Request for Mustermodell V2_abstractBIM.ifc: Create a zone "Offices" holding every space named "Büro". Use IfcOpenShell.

First a look at what the model holds.

```python
import ifcopenshell

model = ifcopenshell.open("Mustermodell V2_abstractBIM.ifc")
print(model.schema)
seen = {}
for space in model.by_type("IfcSpace"):
    seen[space.LongName] = seen.get(space.LongName, 0) + 1
for name, count in sorted(seen.items(), key=str):
    print(count, "x", name)
print("zones:", [z.Name for z in model.by_type("IfcZone")][:20])
```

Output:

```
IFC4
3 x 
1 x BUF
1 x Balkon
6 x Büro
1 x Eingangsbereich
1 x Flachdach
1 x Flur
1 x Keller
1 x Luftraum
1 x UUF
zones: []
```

```python
import ifcopenshell
import ifcopenshell.api.group
import ifcopenshell.api.root

model = ifcopenshell.open("Mustermodell V2_abstractBIM.ifc")

names = {"Büro"}
spaces = [s for s in model.by_type("IfcSpace") if s.LongName in names]

zone = ifcopenshell.api.root.create_entity(model, ifc_class="IfcZone", name="Offices")
ifcopenshell.api.group.assign_group(model, products=spaces, group=zone)
print(len(spaces), "spaces in", zone.Name)

model.write("Mustermodell V2_abstractBIM_rev.ifc")
```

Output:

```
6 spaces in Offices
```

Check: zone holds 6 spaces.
